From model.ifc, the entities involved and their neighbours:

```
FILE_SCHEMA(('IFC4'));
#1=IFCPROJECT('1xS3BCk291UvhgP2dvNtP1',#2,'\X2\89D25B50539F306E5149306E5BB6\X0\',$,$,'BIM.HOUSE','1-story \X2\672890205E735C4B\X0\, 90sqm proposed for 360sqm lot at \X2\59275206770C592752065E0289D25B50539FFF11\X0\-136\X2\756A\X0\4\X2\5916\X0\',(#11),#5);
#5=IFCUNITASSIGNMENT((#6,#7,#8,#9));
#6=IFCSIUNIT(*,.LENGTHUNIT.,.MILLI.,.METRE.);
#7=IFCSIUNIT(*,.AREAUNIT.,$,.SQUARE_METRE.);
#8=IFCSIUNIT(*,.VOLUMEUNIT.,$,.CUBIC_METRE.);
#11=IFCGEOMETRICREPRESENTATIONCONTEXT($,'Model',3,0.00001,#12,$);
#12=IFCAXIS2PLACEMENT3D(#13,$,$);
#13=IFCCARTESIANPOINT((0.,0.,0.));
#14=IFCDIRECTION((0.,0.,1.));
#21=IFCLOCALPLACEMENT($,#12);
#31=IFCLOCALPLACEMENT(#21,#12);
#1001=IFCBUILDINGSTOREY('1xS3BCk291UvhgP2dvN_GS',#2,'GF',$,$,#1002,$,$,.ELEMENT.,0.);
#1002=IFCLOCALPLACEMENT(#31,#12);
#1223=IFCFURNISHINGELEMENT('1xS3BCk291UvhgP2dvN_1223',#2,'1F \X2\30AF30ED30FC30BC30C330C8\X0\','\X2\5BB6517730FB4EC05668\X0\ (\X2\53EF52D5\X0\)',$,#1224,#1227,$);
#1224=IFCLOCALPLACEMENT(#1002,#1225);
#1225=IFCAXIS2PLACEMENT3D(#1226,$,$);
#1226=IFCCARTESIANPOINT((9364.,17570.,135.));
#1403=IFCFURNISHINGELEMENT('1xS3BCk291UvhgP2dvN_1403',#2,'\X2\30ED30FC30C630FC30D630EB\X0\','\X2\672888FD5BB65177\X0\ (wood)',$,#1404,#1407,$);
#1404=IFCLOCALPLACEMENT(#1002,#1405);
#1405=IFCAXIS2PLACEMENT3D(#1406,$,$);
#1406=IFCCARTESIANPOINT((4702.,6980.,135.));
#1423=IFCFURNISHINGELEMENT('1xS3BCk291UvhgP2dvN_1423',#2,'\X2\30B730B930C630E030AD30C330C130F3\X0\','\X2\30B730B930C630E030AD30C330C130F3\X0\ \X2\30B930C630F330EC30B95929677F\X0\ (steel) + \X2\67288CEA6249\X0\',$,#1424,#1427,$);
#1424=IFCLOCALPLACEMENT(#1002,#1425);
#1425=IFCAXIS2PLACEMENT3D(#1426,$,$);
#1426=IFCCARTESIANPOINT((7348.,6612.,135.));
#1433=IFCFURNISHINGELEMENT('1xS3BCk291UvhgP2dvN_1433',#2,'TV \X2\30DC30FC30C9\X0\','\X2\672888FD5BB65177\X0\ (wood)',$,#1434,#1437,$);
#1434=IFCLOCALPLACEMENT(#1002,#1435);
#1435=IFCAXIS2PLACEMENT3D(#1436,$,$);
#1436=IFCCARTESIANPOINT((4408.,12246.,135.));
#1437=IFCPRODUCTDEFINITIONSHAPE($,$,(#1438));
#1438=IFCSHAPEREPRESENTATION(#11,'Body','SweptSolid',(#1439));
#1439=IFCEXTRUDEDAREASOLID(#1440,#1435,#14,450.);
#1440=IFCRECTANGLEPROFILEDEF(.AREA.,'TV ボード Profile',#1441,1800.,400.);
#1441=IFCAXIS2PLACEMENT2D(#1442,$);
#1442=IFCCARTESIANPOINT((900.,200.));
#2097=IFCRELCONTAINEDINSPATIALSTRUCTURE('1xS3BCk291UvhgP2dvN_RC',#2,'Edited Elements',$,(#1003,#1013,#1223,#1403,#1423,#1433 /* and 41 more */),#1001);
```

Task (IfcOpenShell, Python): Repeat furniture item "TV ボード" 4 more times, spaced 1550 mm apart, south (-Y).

```python
import numpy as np
import ifcopenshell
import ifcopenshell.api.geometry
import ifcopenshell.api.root
import ifcopenshell.util.element
import ifcopenshell.util.placement
import ifcopenshell.util.unit

model = ifcopenshell.open("model.ifc")
unit_scale = ifcopenshell.util.unit.calculate_unit_scale(model)


def reuse_history(source, copy):
    """copy_class also copies each property set's owner history, people and application; keep the originals."""
    for rel in copy.IsDefinedBy:
        if rel.is_a("IfcRelDefinesByProperties") and (history := rel.RelatingPropertyDefinition.OwnerHistory):
            rel.RelatingPropertyDefinition.OwnerHistory = source.OwnerHistory
            ifcopenshell.util.element.remove_deep2(model, history)


source = model.by_guid("1xS3BCk291UvhgP2dvN_1433")
base = ifcopenshell.util.placement.get_local_placement(source.ObjectPlacement)
step = np.array([0.0, -1.0, 0.0]) * 1.55 / unit_scale

for i in range(1, 5):
    copy = ifcopenshell.api.root.copy_class(model, product=source)
    copy.Representation = ifcopenshell.util.element.copy_deep(
        model, source.Representation, exclude=["IfcGeometricRepresentationContext", "IfcRepresentationMap"]
    )
    reuse_history(source, copy)
    matrix = base.copy()
    matrix[:3, 3] += i * step
    print("added at", matrix[:3, 3].round(3) + 0.0)
    ifcopenshell.api.geometry.edit_object_placement(model, product=copy, matrix=matrix, is_si=False)

model.write("model_rev.ifc")
```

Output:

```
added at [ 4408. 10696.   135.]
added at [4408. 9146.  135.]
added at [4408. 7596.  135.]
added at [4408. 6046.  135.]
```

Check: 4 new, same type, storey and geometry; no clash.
